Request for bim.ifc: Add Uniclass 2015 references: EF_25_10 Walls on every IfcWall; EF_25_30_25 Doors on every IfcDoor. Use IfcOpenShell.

First a look at what the model holds.

```python
import ifcopenshell

model = ifcopenshell.open("bim.ifc")
print(model.schema)
print("classifications:", [c.Name for c in model.by_type("IfcClassification")])
for ifc_class in ("IfcDoor", "IfcRoof", "IfcStair", "IfcWall", "IfcWindow"):
    print(ifc_class, len(model.by_type(ifc_class)))
```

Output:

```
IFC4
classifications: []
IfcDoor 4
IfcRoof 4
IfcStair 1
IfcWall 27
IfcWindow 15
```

```python
import ifcopenshell
import ifcopenshell.api.classification

model = ifcopenshell.open("bim.ifc")

system = ifcopenshell.api.classification.add_classification(model, classification="Uniclass 2015")

codes = {
    "IfcWall": ("EF_25_10", "Walls"),
    "IfcDoor": ("EF_25_30_25", "Doors"),
}
for ifc_class, (code, name) in codes.items():
    products = model.by_type(ifc_class)
    ifcopenshell.api.classification.add_reference(
        model, products=products, classification=system, identification=code, name=name
    )
    print(code, len(products))

model.write("bim-out.ifc")
```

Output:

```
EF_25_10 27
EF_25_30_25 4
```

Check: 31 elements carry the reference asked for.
